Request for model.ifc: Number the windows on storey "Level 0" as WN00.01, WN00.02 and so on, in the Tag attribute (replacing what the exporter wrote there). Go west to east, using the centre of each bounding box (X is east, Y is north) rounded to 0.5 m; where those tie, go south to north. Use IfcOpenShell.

First a look at what the model holds.

```python
import ifcopenshell
import ifcopenshell.util.element
import ifcopenshell.util.placement

model = ifcopenshell.open("model.ifc")
print(model.schema)
storey = next(s for s in model.by_type("IfcBuildingStorey") if s.Name == "Level 0")
windows = [e for e in ifcopenshell.util.element.get_decomposition(storey) if e.is_a("IfcWindow")]
for e in sorted(windows, key=lambda e: e.id()):
    origin = ifcopenshell.util.placement.get_local_placement(e.ObjectPlacement)[:3, 3]
    print(e.id(), e.Tag, e.Name, origin.round(2) + 0.0, sep=" | ")
```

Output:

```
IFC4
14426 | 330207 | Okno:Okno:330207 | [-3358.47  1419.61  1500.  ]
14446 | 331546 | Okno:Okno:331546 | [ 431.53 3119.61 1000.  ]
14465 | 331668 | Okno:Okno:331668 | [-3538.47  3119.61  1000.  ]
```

```python
import ifcopenshell
import ifcopenshell.geom
import ifcopenshell.util.element
import ifcopenshell.util.shape

model = ifcopenshell.open("model.ifc")
settings = ifcopenshell.geom.settings()
settings.set("use-world-coords", True)


def centre(element):
    shape = ifcopenshell.geom.create_shape(settings, element)
    return ifcopenshell.util.shape.get_bbox_centroid(shape.geometry)


storey = next(s for s in model.by_type("IfcBuildingStorey") if s.Name == "Level 0")
windows = [e for e in ifcopenshell.util.element.get_decomposition(storey) if e.is_a("IfcWindow")]

# Insertion points can sit at a corner or the storey origin, so sort by the geometry (in metres).
centres = {e: centre(e) for e in windows}
windows.sort(key=lambda e: (round(centres[e][0] / 0.5), centres[e][1]))

for i, e in enumerate(windows, start=1):
    number = f"WN00.{i:02d}"
    e.Tag = number
    print(e.id(), number)

model.write("model-out.ifc")
```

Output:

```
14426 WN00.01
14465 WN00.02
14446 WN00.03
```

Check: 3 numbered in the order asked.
